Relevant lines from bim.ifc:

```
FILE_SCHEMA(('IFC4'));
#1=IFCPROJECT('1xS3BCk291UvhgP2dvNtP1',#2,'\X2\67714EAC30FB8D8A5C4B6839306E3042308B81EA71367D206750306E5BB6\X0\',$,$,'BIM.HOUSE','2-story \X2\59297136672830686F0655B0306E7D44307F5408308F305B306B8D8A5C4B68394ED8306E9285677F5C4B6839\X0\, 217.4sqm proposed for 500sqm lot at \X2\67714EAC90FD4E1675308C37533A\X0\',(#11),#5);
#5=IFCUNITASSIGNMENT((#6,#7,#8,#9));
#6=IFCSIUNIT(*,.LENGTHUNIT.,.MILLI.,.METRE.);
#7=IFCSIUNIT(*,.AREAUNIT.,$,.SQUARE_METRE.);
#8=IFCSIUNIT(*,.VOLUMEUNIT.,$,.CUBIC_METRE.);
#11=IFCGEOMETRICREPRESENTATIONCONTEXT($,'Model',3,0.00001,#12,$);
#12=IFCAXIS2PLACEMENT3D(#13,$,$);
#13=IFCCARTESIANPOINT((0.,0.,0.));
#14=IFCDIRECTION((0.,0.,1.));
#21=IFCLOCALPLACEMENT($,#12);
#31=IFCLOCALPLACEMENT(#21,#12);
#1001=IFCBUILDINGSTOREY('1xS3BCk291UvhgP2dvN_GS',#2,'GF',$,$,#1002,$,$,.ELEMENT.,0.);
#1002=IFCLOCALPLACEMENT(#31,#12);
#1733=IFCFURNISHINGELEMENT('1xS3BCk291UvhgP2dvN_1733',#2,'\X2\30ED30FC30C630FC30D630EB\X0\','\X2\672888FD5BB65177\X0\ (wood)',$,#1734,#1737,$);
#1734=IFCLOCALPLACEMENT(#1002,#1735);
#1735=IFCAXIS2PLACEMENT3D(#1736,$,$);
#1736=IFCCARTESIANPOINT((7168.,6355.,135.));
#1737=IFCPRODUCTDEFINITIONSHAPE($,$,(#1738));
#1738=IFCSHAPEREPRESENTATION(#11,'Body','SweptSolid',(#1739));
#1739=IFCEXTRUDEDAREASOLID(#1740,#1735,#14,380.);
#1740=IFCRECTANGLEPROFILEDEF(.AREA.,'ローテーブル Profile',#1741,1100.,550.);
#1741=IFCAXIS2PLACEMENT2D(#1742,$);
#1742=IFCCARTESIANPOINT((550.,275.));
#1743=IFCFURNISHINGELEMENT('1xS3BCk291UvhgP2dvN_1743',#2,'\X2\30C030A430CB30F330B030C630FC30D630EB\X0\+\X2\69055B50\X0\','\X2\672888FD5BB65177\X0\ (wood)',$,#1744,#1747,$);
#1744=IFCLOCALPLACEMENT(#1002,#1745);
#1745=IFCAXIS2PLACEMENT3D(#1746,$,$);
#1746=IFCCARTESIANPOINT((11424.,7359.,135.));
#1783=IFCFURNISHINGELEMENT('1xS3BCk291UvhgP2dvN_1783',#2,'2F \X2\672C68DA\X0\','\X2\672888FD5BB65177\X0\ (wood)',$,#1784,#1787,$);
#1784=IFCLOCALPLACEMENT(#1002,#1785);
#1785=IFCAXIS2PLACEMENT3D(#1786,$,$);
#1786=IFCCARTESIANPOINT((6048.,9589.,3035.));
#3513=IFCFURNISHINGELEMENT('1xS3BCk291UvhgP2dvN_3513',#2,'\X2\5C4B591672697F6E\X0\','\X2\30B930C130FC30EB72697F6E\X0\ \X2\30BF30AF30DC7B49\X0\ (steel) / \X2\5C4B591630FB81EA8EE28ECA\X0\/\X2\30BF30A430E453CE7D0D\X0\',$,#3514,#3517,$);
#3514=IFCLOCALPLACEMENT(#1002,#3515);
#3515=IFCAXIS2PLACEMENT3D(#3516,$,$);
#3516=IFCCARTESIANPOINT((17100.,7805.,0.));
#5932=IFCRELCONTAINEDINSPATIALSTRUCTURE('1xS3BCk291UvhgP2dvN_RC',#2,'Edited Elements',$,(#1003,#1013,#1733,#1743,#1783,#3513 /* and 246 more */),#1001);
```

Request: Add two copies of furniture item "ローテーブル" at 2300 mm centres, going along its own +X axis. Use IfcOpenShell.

```python
import ifcopenshell
import ifcopenshell.api.geometry
import ifcopenshell.api.root
import ifcopenshell.util.element
import ifcopenshell.util.placement

model = ifcopenshell.open("bim.ifc")


def reuse_history(source, copy):
    """copy_class also copies each property set's owner history, people and application; keep the originals."""
    for rel in copy.IsDefinedBy:
        if rel.is_a("IfcRelDefinesByProperties") and (history := rel.RelatingPropertyDefinition.OwnerHistory):
            rel.RelatingPropertyDefinition.OwnerHistory = source.OwnerHistory
            ifcopenshell.util.element.remove_deep2(model, history)


source = model.by_guid("1xS3BCk291UvhgP2dvN_1733")
base = ifcopenshell.util.placement.get_local_placement(source.ObjectPlacement)
step = base[:3, 0] * 2300.0

for i in range(1, 3):
    copy = ifcopenshell.api.root.copy_class(model, product=source)
    copy.Representation = ifcopenshell.util.element.copy_deep(
        model, source.Representation, exclude=["IfcGeometricRepresentationContext", "IfcRepresentationMap"]
    )
    reuse_history(source, copy)
    matrix = base.copy()
    matrix[:3, 3] += i * step
    print("added at", matrix[:3, 3].round(3) + 0.0)
    ifcopenshell.api.geometry.edit_object_placement(model, product=copy, matrix=matrix, is_si=False)

model.write("bim_updated.ifc")
```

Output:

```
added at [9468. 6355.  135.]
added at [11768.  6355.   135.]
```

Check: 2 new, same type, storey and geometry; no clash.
